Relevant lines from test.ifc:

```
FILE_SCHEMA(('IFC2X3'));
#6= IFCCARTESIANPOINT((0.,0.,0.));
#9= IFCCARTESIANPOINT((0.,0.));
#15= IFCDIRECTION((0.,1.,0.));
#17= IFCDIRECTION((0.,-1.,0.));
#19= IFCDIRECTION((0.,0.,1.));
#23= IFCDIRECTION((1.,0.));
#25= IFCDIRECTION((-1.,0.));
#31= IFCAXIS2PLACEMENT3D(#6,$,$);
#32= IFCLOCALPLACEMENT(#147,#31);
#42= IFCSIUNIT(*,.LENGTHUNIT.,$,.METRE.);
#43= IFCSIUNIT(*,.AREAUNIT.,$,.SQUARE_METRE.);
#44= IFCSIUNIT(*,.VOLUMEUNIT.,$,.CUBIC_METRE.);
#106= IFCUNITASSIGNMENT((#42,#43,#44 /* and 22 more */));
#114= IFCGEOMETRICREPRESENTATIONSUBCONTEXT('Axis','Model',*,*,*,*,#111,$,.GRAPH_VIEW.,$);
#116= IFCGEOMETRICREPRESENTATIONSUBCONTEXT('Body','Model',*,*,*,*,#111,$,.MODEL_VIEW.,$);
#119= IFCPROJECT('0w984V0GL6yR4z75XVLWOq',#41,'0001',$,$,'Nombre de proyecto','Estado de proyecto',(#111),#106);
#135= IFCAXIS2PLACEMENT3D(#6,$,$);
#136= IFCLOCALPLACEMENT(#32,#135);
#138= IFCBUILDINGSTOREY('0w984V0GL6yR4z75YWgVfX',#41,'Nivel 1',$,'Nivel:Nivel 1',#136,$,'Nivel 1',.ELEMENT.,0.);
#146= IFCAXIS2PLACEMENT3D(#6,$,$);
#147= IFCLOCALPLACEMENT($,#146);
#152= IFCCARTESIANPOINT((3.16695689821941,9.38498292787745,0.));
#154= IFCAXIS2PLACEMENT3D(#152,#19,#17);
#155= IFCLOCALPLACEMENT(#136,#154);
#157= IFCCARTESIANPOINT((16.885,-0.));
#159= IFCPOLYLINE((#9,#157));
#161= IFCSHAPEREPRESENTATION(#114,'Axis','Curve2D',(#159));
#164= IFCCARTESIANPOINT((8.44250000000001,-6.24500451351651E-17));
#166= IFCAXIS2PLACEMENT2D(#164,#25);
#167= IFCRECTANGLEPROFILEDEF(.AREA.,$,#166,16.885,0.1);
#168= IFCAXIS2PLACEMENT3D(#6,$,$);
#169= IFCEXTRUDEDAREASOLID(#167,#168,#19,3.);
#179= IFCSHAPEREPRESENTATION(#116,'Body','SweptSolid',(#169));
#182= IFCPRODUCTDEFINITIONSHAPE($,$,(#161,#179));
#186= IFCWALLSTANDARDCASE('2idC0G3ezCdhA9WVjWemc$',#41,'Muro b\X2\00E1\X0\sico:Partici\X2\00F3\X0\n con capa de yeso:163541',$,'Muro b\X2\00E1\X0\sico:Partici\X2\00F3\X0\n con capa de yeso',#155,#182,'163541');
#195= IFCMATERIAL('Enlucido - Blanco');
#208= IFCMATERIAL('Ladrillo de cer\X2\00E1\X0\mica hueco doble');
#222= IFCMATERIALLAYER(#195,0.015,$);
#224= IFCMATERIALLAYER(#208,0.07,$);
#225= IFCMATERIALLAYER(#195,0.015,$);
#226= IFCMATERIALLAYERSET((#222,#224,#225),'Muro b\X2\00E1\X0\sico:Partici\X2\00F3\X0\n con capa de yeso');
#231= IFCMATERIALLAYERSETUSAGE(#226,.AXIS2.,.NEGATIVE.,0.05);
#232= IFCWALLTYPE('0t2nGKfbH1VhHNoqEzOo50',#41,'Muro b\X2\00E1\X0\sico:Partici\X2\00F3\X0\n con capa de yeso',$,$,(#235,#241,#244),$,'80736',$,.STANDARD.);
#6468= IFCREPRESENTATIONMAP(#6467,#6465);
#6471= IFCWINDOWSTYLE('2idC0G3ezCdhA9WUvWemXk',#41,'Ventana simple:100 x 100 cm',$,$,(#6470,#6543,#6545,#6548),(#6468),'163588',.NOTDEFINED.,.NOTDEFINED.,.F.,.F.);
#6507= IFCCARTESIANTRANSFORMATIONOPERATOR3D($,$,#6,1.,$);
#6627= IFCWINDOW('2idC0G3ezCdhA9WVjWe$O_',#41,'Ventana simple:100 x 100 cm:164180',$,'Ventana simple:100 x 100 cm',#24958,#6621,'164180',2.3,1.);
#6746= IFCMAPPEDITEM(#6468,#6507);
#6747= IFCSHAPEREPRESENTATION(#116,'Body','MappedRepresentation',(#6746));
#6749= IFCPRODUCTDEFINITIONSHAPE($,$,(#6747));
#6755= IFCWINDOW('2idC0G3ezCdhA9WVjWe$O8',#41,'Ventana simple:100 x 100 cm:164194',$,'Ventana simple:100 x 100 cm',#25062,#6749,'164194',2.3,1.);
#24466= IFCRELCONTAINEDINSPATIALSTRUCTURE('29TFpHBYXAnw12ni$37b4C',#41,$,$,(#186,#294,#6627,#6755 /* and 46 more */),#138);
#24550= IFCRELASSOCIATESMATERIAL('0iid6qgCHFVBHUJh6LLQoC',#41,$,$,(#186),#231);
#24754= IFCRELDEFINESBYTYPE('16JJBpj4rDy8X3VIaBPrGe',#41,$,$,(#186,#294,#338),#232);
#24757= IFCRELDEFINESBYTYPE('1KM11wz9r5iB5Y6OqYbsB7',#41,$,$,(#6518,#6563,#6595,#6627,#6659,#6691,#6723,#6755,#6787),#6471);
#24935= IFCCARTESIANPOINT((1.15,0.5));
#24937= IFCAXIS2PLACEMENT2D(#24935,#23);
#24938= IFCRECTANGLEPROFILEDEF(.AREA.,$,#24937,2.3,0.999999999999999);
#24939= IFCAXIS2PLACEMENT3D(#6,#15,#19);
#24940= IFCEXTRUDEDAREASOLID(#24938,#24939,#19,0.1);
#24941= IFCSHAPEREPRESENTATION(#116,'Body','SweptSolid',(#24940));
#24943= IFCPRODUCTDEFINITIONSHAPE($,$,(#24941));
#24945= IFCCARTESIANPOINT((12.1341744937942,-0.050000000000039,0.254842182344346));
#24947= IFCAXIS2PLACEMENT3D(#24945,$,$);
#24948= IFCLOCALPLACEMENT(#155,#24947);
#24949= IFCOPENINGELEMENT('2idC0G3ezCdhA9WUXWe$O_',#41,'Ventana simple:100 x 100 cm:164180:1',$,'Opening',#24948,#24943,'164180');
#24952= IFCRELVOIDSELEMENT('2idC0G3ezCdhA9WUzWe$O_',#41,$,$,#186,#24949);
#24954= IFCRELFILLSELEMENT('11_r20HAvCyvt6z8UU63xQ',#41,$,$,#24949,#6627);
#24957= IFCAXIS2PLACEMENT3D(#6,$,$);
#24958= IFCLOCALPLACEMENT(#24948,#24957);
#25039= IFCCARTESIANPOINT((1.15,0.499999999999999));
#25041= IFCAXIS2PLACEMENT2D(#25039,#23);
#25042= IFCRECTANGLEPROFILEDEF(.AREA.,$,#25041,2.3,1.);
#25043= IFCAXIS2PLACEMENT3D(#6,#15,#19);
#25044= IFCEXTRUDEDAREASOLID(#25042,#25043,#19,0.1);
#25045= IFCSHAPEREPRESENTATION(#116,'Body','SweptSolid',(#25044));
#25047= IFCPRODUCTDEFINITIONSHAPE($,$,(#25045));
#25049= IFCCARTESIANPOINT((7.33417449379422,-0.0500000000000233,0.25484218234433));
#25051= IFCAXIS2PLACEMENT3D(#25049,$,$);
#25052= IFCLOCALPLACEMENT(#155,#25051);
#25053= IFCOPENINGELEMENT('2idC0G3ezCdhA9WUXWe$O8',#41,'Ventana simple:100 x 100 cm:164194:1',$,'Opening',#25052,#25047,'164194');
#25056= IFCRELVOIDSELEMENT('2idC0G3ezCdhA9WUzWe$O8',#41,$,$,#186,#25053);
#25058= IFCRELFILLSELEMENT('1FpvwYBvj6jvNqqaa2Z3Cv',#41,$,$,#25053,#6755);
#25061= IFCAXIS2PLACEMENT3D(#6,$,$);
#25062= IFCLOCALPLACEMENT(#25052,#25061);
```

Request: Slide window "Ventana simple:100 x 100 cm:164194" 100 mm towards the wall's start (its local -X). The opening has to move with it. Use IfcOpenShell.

```python
import ifcopenshell
import ifcopenshell.api.geometry
import ifcopenshell.util.placement

model = ifcopenshell.open("test.ifc")

window = model.by_guid("2idC0G3ezCdhA9WVjWe$O8")
opening = window.FillsVoids[0].RelatingOpeningElement
wall = opening.VoidsElements[0].RelatingBuildingElement

wall_matrix = ifcopenshell.util.placement.get_local_placement(wall.ObjectPlacement)
shift = wall_matrix[:3, 0] * -0.1
before = ifcopenshell.util.placement.get_local_placement(window.ObjectPlacement)[:3, 3].copy()

# The window is placed relative to its opening, so it follows when the opening moves.
matrix = ifcopenshell.util.placement.get_local_placement(opening.ObjectPlacement)
matrix[:3, 3] += shift
ifcopenshell.api.geometry.edit_object_placement(
    model, product=opening, matrix=matrix, is_si=False, should_transform_children=True
)

after = ifcopenshell.util.placement.get_local_placement(window.ObjectPlacement)[:3, 3]
print("window moved by", (after - before).round(3) + 0.0)

model.write("test_v2.ifc")
```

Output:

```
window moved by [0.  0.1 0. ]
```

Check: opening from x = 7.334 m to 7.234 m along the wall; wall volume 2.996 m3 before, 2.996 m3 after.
